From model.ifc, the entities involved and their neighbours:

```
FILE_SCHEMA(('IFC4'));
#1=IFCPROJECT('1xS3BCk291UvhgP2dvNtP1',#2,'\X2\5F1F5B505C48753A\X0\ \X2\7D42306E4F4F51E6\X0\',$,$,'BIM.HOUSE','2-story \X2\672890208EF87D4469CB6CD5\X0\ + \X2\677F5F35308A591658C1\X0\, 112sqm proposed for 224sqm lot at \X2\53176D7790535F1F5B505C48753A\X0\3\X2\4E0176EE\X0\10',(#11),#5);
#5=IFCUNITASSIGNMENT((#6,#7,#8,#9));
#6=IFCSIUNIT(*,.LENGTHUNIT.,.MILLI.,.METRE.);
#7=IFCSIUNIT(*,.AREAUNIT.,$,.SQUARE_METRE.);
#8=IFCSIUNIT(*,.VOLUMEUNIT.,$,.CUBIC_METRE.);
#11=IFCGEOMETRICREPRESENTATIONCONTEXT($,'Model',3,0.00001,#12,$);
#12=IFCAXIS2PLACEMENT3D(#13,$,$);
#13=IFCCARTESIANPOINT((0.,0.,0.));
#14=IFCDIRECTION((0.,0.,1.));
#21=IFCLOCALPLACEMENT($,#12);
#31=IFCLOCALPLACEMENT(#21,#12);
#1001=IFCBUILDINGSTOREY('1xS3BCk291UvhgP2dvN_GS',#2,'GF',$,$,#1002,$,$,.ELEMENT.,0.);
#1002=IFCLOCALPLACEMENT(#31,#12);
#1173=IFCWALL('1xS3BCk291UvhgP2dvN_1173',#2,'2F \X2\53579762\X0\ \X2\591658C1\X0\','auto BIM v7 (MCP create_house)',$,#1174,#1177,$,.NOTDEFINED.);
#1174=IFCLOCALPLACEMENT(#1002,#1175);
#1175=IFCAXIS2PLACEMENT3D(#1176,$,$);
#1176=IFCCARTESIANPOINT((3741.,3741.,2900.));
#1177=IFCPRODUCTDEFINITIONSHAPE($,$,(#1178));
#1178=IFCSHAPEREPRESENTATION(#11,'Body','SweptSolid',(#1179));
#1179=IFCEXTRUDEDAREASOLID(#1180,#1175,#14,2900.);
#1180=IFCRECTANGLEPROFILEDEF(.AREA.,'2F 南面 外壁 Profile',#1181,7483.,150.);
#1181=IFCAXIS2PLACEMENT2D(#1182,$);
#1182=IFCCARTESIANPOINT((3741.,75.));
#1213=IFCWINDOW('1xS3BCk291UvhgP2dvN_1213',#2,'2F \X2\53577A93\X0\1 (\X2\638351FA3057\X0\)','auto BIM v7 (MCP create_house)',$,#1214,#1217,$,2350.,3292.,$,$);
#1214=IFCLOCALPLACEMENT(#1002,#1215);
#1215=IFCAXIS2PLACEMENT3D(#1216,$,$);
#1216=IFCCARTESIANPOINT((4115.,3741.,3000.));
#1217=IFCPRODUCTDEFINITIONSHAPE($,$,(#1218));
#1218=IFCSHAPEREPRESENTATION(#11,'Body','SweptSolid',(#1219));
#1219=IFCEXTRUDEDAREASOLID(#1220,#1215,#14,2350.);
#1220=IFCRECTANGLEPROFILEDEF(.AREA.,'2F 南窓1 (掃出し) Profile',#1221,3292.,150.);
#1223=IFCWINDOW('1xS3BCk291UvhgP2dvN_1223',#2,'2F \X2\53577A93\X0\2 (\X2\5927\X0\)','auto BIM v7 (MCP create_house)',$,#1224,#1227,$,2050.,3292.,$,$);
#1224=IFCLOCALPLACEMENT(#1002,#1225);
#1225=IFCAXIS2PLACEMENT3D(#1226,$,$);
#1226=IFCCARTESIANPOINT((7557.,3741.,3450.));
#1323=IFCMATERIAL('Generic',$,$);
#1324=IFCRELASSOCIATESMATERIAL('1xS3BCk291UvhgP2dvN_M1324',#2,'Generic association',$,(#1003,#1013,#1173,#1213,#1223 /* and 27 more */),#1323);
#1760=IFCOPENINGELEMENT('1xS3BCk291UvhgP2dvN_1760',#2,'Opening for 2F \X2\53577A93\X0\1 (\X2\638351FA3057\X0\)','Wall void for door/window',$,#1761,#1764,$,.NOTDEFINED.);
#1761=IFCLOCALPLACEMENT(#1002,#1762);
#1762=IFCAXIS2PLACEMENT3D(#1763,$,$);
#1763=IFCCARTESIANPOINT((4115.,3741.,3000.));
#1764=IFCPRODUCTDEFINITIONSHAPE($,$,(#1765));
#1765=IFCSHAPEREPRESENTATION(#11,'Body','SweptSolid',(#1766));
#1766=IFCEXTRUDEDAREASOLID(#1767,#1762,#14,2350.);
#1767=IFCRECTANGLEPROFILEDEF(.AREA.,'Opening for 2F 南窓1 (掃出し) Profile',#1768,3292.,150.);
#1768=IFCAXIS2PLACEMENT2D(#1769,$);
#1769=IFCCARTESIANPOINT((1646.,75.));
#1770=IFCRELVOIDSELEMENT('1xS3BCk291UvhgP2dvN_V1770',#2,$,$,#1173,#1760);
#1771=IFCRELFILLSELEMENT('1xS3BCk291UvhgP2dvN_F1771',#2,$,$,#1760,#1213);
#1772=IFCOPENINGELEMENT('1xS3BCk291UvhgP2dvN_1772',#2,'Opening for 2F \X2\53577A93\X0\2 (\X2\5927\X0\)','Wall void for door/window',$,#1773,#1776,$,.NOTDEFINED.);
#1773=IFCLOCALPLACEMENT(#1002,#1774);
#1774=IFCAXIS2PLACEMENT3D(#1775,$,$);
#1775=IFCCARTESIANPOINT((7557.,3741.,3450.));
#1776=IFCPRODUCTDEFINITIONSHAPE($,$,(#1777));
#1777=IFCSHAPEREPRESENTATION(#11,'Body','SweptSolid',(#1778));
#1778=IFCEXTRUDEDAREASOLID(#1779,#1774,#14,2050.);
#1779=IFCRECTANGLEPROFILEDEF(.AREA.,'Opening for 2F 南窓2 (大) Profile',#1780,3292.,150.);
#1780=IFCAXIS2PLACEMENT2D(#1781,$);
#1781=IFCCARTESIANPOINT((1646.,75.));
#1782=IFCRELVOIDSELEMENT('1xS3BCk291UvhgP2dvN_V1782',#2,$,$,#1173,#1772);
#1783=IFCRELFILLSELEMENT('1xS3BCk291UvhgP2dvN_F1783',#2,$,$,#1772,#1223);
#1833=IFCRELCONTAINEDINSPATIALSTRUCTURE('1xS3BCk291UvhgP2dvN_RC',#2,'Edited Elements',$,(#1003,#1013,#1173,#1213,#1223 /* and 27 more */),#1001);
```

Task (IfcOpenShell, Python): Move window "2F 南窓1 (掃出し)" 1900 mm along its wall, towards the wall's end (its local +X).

```python
import ifcopenshell
import ifcopenshell.api.geometry
import ifcopenshell.util.placement
import ifcopenshell.util.unit

model = ifcopenshell.open("model.ifc")
unit_scale = ifcopenshell.util.unit.calculate_unit_scale(model)

window = model.by_id(1213)
opening = window.FillsVoids[0].RelatingOpeningElement
wall = opening.VoidsElements[0].RelatingBuildingElement

wall_matrix = ifcopenshell.util.placement.get_local_placement(wall.ObjectPlacement)
shift = wall_matrix[:3, 0] * 1.9 / unit_scale
before = ifcopenshell.util.placement.get_local_placement(window.ObjectPlacement)[:3, 3].copy()

# The window is not placed relative to its opening, so move both.
for product in (opening, window):
    matrix = ifcopenshell.util.placement.get_local_placement(product.ObjectPlacement)
    matrix[:3, 3] += shift
    ifcopenshell.api.geometry.edit_object_placement(model, product=product, matrix=matrix, is_si=False)

after = ifcopenshell.util.placement.get_local_placement(window.ObjectPlacement)[:3, 3]
print("window moved by", (after - before).round(3) + 0.0)

model.write("model_rev.ifc")
```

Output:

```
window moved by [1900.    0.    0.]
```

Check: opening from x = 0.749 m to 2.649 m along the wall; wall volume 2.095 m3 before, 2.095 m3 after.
